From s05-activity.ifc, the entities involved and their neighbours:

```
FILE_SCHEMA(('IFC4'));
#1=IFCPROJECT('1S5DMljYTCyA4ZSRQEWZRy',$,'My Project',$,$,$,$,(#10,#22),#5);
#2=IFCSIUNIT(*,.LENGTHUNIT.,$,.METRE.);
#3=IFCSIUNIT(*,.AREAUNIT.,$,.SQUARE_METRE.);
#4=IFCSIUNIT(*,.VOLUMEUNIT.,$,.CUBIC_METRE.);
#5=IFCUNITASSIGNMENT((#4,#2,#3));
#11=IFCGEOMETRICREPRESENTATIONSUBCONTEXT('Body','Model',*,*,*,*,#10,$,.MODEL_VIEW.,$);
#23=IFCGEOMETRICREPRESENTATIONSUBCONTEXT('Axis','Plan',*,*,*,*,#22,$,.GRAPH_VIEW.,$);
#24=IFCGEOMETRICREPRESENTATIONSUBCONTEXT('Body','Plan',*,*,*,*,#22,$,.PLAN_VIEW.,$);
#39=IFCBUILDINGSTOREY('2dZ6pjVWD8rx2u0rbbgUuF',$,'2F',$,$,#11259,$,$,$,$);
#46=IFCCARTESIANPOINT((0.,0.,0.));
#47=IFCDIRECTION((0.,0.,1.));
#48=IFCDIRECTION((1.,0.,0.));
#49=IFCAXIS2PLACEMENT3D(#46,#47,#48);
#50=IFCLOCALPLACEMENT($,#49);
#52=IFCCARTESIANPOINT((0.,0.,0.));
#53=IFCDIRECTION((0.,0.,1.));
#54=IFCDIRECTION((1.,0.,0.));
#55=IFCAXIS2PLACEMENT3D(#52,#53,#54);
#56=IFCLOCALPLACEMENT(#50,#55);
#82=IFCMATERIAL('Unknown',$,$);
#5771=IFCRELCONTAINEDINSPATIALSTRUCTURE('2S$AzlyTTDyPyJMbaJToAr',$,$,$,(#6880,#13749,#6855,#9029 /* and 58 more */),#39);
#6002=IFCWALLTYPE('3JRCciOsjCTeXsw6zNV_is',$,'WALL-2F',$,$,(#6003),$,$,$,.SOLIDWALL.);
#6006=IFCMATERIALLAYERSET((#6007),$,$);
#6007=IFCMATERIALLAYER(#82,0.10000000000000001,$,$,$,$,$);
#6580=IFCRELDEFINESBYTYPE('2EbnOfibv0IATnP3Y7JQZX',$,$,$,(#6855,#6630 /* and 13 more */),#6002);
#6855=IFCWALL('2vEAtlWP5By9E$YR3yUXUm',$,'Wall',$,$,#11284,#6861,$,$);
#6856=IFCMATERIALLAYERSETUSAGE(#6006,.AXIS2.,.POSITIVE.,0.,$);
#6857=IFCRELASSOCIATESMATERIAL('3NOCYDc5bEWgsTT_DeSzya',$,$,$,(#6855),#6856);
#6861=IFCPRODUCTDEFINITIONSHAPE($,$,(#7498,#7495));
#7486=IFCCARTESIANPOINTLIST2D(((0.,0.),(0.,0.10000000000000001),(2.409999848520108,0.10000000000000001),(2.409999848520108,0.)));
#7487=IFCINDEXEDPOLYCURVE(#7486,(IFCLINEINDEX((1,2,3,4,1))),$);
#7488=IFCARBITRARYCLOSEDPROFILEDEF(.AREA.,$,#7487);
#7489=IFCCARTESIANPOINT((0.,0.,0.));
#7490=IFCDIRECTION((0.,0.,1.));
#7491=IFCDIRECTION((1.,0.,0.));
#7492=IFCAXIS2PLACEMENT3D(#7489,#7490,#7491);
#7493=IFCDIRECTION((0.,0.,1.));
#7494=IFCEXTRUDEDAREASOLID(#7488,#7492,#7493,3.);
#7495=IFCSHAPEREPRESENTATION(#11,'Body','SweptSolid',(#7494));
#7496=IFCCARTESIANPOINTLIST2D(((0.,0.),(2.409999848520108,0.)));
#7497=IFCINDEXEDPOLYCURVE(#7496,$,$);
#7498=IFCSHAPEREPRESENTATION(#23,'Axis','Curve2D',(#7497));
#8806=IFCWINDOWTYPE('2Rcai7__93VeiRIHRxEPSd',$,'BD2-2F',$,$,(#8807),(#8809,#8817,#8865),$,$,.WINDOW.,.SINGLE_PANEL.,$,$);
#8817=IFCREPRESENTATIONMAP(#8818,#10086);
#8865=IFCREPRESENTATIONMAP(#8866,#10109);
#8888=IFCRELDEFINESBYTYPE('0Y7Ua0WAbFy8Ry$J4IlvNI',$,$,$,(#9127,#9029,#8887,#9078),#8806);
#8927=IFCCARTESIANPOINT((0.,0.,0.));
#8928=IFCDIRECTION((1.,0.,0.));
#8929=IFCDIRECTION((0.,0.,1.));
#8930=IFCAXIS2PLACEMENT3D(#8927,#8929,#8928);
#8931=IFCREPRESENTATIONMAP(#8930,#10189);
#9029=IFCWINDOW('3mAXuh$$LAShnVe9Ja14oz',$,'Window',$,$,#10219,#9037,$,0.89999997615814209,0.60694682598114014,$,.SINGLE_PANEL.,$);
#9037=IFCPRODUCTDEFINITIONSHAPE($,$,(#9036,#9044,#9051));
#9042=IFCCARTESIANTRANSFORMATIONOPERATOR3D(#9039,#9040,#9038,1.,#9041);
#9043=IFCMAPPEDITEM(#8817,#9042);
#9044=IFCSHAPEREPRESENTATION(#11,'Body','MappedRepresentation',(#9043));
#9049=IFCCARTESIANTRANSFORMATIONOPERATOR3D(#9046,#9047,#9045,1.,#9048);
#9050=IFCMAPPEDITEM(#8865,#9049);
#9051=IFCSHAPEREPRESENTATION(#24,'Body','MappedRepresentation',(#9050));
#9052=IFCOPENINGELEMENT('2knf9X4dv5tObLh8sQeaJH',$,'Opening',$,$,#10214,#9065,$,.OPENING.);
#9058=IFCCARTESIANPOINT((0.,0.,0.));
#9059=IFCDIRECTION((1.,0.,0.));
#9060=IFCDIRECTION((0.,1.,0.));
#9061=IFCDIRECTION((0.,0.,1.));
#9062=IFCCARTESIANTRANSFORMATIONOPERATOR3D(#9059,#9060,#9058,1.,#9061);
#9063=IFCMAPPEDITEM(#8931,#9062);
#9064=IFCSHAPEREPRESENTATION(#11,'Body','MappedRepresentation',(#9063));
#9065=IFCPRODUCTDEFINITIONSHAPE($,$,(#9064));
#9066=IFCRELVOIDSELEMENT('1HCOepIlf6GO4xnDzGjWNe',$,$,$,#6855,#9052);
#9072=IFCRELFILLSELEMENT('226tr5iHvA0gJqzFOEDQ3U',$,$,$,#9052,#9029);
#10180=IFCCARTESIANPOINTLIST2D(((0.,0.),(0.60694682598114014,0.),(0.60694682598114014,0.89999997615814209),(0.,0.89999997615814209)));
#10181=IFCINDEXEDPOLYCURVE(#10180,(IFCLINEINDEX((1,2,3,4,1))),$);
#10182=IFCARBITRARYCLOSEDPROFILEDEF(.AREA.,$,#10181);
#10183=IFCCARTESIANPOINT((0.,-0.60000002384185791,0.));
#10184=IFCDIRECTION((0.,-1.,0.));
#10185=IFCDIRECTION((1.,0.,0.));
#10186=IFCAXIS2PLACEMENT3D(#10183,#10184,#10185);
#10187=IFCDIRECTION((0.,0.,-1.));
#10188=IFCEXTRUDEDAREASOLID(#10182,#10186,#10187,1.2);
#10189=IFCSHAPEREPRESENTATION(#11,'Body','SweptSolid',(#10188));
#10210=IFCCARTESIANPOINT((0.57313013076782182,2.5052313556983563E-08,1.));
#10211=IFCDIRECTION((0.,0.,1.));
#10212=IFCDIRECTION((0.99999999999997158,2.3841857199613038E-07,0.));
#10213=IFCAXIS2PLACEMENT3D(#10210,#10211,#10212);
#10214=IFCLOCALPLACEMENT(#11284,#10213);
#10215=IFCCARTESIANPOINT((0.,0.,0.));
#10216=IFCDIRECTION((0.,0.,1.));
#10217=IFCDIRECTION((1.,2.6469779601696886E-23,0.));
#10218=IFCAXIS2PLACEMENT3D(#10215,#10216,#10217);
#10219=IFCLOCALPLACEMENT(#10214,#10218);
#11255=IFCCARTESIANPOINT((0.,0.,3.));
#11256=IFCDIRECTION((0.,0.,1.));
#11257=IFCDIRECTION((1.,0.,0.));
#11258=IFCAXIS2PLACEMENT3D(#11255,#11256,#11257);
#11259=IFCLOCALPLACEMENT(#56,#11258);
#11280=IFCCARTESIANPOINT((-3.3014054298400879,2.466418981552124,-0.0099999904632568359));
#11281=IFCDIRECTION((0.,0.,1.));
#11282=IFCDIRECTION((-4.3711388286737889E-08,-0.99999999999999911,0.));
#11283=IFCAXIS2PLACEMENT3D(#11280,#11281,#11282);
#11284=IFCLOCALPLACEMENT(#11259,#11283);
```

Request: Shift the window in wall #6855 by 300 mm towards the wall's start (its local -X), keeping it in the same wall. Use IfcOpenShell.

```python
import ifcopenshell
import ifcopenshell.api.geometry
import ifcopenshell.util.placement
import ifcopenshell.util.unit

model = ifcopenshell.open("s05-activity.ifc")
unit_scale = ifcopenshell.util.unit.calculate_unit_scale(model)

window = model.by_guid("3mAXuh$$LAShnVe9Ja14oz")
opening = window.FillsVoids[0].RelatingOpeningElement
wall = opening.VoidsElements[0].RelatingBuildingElement

wall_matrix = ifcopenshell.util.placement.get_local_placement(wall.ObjectPlacement)
shift = wall_matrix[:3, 0] * -0.3 / unit_scale
before = ifcopenshell.util.placement.get_local_placement(window.ObjectPlacement)[:3, 3].copy()

# The window is placed relative to its opening, so it follows when the opening moves.
matrix = ifcopenshell.util.placement.get_local_placement(opening.ObjectPlacement)
matrix[:3, 3] += shift
ifcopenshell.api.geometry.edit_object_placement(
    model, product=opening, matrix=matrix, is_si=False, should_transform_children=True
)

after = ifcopenshell.util.placement.get_local_placement(window.ObjectPlacement)[:3, 3]
print("window moved by", (after - before).round(3) + 0.0)

model.write("s05-activity_edited.ifc")
```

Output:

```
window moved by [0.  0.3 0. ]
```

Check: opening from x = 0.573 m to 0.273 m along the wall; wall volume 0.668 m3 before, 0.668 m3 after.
